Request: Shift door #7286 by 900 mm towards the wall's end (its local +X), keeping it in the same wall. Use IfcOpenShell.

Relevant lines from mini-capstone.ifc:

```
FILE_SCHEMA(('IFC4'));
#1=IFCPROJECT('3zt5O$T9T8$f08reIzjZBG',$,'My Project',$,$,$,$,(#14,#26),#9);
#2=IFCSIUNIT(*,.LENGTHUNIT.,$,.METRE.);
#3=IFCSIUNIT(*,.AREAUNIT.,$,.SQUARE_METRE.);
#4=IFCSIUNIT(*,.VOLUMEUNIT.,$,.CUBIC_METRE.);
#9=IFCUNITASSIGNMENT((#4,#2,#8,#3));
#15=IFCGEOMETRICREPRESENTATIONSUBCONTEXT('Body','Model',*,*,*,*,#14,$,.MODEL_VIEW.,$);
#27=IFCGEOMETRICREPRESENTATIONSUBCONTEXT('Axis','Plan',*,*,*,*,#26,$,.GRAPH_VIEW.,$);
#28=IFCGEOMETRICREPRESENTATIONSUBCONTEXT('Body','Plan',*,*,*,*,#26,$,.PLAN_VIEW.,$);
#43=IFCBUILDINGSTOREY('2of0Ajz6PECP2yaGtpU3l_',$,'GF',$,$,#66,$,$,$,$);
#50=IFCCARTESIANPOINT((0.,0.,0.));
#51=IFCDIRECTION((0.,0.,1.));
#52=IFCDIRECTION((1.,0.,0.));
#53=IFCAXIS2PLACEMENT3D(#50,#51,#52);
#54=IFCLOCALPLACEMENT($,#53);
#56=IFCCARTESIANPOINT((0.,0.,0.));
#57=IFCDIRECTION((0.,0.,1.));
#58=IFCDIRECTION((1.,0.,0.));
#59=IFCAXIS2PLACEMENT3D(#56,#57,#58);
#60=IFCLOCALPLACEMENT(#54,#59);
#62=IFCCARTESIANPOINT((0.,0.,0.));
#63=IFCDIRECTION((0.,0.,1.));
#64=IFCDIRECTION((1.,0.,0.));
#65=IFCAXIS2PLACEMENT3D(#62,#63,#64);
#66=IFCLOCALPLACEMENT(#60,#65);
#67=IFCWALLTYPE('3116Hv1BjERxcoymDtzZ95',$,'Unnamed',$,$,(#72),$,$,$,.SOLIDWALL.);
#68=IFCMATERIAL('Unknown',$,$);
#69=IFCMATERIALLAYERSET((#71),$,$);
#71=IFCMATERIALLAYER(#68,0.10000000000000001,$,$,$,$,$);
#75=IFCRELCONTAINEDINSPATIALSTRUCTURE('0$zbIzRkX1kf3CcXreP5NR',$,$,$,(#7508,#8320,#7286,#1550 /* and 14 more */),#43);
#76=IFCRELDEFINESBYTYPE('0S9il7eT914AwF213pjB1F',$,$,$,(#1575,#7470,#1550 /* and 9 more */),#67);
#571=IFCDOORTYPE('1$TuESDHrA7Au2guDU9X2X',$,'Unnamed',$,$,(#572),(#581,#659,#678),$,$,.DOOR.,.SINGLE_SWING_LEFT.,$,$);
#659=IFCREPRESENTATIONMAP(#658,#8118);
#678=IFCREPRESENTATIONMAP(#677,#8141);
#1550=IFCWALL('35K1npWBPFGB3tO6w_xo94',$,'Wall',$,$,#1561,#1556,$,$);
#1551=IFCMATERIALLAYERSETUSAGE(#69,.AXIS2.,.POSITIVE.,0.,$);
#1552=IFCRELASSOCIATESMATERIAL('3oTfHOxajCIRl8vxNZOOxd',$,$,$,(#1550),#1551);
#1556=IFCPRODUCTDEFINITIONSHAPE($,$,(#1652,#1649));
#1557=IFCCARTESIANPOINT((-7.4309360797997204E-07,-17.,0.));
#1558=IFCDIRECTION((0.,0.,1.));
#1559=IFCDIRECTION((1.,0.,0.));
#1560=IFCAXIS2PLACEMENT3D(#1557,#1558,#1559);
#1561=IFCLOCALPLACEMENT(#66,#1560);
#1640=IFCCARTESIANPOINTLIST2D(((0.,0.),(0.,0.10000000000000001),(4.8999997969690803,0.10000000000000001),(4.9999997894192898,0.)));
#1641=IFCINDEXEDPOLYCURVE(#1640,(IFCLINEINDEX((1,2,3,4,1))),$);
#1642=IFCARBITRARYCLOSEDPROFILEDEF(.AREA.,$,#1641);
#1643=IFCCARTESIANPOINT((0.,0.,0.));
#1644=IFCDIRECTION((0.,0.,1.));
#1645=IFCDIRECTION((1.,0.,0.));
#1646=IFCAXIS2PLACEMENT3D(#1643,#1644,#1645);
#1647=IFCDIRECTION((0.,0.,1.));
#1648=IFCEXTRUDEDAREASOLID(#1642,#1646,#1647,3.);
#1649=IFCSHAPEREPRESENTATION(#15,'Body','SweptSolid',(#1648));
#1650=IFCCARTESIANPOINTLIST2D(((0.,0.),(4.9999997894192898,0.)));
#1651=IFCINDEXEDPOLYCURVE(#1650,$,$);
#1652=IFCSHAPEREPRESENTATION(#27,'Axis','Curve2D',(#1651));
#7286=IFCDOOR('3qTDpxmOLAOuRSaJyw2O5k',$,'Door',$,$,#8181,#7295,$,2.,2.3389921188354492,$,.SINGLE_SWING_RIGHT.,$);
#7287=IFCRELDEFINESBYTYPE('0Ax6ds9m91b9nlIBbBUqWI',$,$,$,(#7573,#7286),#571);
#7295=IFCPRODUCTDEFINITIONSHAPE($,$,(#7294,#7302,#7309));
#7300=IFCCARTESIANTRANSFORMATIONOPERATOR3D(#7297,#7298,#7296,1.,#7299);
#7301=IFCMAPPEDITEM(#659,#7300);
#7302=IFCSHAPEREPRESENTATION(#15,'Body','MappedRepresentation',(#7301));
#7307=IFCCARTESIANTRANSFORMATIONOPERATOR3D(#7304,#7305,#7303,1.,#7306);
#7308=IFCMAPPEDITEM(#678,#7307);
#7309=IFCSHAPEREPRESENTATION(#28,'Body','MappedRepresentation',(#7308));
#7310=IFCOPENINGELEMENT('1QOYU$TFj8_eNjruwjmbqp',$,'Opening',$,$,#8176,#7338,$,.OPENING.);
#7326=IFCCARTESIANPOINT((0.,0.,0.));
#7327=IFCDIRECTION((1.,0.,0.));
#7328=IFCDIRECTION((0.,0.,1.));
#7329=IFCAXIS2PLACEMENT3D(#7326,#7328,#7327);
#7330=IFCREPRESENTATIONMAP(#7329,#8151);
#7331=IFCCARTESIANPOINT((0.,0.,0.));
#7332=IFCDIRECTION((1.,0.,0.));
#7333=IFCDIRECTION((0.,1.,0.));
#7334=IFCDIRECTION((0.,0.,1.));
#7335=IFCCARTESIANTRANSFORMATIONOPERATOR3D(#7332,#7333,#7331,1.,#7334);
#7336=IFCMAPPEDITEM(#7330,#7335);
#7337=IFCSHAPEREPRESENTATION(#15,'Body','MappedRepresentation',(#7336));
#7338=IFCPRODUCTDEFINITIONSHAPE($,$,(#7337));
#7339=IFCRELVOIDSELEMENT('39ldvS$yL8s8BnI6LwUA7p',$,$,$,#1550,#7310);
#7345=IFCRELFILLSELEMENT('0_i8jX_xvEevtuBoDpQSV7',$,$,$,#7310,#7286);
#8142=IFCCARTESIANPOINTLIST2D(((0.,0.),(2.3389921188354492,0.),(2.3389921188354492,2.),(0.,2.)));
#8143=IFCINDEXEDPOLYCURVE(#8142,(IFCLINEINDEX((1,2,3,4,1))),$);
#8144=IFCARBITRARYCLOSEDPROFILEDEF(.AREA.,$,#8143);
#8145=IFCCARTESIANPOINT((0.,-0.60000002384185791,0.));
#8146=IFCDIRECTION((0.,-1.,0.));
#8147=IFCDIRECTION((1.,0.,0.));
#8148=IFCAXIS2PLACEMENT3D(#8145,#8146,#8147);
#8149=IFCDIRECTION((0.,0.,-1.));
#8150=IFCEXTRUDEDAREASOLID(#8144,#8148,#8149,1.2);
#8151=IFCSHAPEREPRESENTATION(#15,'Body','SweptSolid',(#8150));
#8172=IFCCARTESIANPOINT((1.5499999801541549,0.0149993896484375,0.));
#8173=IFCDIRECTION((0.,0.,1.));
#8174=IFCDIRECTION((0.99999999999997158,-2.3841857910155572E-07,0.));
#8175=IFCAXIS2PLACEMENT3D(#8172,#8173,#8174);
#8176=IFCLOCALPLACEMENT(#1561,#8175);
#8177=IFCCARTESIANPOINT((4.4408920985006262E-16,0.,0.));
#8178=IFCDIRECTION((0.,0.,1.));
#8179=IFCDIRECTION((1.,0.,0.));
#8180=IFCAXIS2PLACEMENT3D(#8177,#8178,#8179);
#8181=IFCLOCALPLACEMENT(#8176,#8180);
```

```python
import ifcopenshell
import ifcopenshell.api.geometry
import ifcopenshell.util.placement
import ifcopenshell.util.unit

model = ifcopenshell.open("mini-capstone.ifc")
unit_scale = ifcopenshell.util.unit.calculate_unit_scale(model)

door = model.by_guid("3qTDpxmOLAOuRSaJyw2O5k")
opening = door.FillsVoids[0].RelatingOpeningElement
wall = opening.VoidsElements[0].RelatingBuildingElement

wall_matrix = ifcopenshell.util.placement.get_local_placement(wall.ObjectPlacement)
shift = wall_matrix[:3, 0] * 0.9 / unit_scale
before = ifcopenshell.util.placement.get_local_placement(door.ObjectPlacement)[:3, 3].copy()

# The door is placed relative to its opening, so it follows when the opening moves.
matrix = ifcopenshell.util.placement.get_local_placement(opening.ObjectPlacement)
matrix[:3, 3] += shift
ifcopenshell.api.geometry.edit_object_placement(
    model, product=opening, matrix=matrix, is_si=False, should_transform_children=True
)

after = ifcopenshell.util.placement.get_local_placement(door.ObjectPlacement)[:3, 3]
print("door moved by", (after - before).round(3) + 0.0)

model.write("mini-capstone_edited.ifc")
```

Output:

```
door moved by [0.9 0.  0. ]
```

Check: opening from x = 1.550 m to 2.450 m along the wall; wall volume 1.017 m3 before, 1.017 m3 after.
